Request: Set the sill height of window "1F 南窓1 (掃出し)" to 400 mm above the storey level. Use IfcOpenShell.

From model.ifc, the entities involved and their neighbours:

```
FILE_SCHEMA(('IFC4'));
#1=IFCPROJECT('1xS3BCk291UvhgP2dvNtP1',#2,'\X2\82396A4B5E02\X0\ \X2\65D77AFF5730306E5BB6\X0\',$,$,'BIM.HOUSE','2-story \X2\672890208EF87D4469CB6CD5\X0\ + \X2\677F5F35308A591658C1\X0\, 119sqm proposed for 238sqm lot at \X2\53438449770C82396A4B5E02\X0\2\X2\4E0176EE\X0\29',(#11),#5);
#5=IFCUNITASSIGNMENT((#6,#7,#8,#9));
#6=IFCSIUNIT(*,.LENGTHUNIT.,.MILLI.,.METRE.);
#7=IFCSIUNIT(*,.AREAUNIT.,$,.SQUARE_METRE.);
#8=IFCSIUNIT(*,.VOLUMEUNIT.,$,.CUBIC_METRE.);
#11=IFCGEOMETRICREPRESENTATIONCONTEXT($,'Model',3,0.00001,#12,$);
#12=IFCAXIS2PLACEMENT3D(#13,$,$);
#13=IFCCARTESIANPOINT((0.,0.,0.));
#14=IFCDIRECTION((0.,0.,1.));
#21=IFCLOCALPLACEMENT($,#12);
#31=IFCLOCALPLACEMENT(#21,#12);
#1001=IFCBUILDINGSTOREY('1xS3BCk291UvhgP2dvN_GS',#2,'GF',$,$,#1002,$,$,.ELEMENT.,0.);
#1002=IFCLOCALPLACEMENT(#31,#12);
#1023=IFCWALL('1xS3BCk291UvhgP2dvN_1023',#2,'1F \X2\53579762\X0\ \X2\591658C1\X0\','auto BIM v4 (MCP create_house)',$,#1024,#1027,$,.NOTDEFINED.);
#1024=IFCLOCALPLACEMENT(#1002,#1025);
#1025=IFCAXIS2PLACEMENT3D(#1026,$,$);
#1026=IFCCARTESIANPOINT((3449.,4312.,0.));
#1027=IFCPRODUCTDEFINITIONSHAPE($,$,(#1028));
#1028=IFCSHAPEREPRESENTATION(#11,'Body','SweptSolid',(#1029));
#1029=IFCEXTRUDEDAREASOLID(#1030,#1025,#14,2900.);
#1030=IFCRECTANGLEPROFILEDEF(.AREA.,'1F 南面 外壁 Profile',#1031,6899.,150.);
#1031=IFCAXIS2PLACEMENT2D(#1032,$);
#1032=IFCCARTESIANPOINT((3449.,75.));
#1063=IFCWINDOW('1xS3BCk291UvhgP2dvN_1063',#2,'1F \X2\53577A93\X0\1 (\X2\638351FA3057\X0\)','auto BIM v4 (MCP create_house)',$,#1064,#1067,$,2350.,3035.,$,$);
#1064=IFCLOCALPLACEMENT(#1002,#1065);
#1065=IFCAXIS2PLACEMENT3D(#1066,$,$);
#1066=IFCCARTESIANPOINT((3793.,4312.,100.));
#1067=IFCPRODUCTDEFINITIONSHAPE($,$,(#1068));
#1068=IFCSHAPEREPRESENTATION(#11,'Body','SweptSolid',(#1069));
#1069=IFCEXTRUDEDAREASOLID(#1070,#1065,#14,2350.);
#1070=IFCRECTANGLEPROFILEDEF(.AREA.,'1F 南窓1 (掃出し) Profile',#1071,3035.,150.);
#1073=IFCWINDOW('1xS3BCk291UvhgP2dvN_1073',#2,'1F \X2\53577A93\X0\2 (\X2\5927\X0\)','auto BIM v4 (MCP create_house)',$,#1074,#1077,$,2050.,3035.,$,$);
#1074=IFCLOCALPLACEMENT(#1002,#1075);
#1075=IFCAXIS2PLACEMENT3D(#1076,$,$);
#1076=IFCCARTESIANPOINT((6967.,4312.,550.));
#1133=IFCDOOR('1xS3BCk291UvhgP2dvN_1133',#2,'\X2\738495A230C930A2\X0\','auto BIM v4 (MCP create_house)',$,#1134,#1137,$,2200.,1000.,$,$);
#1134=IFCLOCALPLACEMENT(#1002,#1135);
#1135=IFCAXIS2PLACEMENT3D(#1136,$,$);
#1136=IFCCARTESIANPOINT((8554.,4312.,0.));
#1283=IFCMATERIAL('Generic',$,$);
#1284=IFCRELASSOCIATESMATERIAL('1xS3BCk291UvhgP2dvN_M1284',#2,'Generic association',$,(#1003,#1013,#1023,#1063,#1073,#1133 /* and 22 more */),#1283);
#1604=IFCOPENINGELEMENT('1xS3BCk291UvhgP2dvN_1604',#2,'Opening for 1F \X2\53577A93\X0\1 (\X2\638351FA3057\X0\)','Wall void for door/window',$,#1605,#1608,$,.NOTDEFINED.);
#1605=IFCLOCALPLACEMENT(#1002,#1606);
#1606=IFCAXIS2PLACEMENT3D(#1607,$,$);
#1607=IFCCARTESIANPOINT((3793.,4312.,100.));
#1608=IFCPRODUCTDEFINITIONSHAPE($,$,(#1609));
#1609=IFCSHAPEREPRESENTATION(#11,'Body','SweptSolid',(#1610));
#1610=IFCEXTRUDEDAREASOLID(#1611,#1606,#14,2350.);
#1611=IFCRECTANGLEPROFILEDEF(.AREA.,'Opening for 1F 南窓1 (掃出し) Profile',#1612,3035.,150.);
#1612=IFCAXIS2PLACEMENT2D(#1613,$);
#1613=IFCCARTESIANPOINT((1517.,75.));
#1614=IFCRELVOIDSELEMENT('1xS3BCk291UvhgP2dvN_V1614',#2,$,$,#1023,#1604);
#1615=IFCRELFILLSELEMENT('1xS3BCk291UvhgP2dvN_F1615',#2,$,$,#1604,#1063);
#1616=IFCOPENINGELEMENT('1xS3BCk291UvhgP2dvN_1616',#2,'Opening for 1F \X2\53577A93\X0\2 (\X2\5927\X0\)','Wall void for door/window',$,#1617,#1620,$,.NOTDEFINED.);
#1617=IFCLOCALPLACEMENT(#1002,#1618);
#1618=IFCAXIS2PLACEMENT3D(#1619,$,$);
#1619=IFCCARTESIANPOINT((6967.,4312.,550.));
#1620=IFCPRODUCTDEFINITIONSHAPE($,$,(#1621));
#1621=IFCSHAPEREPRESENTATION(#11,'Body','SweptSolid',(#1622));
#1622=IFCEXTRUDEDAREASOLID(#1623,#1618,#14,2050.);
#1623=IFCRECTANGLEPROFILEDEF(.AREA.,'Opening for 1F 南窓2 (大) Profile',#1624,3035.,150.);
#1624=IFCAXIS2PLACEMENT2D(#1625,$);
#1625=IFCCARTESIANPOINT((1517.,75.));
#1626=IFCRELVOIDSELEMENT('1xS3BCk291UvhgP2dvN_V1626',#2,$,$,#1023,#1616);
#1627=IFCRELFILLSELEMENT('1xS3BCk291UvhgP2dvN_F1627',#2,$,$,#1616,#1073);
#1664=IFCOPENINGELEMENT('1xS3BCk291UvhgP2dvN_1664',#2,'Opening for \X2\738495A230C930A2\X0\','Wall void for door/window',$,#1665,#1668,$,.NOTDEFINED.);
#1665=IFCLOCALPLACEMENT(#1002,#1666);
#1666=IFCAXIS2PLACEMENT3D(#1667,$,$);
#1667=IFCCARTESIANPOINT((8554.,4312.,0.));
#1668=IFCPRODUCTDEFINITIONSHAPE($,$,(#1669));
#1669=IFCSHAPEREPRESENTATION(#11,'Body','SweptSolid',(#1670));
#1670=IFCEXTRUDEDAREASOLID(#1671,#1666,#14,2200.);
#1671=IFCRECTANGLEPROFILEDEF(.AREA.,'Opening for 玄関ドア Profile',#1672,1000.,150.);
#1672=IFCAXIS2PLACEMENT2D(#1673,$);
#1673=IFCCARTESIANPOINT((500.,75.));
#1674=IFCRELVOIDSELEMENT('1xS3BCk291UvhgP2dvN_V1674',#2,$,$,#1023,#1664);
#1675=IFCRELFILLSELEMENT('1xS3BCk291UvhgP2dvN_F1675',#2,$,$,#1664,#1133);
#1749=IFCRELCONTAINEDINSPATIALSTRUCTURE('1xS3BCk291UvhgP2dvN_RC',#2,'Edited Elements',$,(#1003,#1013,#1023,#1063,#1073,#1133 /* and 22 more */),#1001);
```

```python
import numpy as np
import ifcopenshell
import ifcopenshell.api.geometry
import ifcopenshell.geom
import ifcopenshell.util.element
import ifcopenshell.util.placement
import ifcopenshell.util.shape
import ifcopenshell.util.unit

model = ifcopenshell.open("model.ifc")
unit_scale = ifcopenshell.util.unit.calculate_unit_scale(model)

window = model.by_id(1063)
opening = window.FillsVoids[0].RelatingOpeningElement
storey = ifcopenshell.util.element.get_container(window, ifc_class="IfcBuildingStorey")
level = ifcopenshell.util.placement.get_local_placement(storey.ObjectPlacement)[2, 3]

# The opening's origin need not be at the sill, so measure its lowest point.
shape = ifcopenshell.geom.create_shape(ifcopenshell.geom.settings(), opening)
bottom = ifcopenshell.util.shape.get_shape_bottom_elevation(shape, shape.geometry) / unit_scale
dz = level + 400.0 - bottom

shift = np.array([0.0, 0.0, dz])
# The window is not placed relative to its opening, so move both.
for product in (opening, window):
    matrix = ifcopenshell.util.placement.get_local_placement(product.ObjectPlacement)
    matrix[:3, 3] += shift
    ifcopenshell.api.geometry.edit_object_placement(model, product=product, matrix=matrix, is_si=False)

print(f"moved by {dz * unit_scale:+.3f} m")

model.write("model_updated.ifc")
```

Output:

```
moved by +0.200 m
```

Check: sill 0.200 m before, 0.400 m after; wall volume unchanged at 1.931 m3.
